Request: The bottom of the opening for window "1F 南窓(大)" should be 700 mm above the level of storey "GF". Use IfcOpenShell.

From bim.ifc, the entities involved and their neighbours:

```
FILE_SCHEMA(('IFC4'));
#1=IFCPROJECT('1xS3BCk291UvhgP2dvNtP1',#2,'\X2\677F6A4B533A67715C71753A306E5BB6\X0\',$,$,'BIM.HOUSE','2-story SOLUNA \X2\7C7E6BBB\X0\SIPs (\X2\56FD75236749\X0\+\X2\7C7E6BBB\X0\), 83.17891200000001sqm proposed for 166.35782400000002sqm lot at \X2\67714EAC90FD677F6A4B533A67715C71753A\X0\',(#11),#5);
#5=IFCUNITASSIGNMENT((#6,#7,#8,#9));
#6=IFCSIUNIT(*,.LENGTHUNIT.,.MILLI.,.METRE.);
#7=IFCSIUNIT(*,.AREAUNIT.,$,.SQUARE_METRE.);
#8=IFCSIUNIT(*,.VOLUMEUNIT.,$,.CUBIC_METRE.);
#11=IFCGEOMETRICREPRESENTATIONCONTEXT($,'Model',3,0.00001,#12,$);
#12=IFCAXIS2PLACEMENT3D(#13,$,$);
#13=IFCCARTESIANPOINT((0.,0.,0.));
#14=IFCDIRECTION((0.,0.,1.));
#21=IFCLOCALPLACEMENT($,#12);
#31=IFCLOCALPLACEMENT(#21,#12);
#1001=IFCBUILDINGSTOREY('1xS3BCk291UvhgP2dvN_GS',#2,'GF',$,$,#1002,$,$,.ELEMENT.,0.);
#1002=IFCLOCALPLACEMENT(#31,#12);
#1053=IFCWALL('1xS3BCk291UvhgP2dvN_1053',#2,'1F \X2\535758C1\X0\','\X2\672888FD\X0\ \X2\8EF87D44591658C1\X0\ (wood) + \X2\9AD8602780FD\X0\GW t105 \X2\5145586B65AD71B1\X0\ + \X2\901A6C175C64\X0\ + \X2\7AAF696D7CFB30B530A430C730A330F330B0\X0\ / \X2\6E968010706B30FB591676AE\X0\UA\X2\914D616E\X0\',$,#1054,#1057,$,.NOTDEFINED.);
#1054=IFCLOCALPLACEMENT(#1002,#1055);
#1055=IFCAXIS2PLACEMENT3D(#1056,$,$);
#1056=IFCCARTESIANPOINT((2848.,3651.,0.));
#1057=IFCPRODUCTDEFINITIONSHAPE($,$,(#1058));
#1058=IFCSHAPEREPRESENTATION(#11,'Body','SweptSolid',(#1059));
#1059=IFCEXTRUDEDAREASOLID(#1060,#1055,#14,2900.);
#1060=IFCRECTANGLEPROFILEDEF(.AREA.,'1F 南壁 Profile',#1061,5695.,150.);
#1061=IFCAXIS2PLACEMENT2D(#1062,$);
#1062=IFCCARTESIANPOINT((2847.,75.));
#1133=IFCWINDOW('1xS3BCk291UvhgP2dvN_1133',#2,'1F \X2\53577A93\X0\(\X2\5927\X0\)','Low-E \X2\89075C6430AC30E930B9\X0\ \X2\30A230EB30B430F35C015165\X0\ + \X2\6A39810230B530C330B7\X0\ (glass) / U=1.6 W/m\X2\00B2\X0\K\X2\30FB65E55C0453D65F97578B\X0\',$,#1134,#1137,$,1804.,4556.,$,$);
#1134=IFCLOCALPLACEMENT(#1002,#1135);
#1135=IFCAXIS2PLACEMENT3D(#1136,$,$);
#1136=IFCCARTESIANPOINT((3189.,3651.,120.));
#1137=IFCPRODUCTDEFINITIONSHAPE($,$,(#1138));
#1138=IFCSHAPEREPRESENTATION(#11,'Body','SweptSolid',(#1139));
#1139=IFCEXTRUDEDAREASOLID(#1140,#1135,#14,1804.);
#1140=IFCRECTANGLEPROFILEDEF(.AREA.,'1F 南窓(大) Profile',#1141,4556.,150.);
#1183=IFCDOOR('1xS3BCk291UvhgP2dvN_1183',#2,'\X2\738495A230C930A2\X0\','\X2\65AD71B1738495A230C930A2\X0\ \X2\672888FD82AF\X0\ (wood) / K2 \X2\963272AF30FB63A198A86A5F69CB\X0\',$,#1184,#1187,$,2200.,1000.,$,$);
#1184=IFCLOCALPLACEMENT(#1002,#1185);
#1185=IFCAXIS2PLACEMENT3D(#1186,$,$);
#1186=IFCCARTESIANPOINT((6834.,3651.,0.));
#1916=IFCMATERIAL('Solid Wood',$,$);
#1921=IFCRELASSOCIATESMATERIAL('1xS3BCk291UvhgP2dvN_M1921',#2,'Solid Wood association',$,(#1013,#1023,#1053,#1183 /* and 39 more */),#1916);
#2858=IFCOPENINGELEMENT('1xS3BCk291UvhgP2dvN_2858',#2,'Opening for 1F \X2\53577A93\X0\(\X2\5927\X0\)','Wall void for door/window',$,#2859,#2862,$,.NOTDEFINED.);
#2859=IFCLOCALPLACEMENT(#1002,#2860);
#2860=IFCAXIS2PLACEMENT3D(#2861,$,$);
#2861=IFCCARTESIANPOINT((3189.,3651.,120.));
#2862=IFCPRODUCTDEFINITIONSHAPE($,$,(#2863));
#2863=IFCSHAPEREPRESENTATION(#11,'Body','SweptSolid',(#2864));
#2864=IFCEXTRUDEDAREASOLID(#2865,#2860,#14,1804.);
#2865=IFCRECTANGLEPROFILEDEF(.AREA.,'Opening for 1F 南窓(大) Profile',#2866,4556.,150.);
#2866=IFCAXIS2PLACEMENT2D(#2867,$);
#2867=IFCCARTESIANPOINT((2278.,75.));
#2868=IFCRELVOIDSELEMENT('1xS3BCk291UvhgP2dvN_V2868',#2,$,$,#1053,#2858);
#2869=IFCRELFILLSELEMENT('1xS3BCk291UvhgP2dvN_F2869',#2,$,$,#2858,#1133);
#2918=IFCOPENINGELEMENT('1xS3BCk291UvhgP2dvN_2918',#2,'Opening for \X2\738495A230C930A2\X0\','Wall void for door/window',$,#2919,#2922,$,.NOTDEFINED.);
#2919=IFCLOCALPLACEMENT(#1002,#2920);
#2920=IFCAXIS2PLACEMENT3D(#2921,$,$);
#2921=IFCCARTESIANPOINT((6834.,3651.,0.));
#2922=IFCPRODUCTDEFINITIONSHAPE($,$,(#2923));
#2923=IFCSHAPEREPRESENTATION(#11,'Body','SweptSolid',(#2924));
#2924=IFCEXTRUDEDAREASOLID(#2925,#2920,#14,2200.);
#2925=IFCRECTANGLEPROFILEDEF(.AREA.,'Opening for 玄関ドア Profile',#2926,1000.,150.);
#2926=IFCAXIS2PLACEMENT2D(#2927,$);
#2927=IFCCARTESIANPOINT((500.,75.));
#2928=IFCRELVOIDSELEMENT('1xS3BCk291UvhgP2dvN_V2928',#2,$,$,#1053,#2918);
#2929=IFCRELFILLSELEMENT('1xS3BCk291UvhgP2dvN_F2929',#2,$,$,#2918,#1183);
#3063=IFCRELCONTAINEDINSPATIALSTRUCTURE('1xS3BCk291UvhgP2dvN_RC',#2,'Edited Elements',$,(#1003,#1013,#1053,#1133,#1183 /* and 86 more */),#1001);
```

```python
import numpy as np
import ifcopenshell
import ifcopenshell.api.geometry
import ifcopenshell.geom
import ifcopenshell.util.element
import ifcopenshell.util.placement
import ifcopenshell.util.shape
import ifcopenshell.util.unit

model = ifcopenshell.open("bim.ifc")
unit_scale = ifcopenshell.util.unit.calculate_unit_scale(model)

window = model.by_guid("1xS3BCk291UvhgP2dvN_1133")
opening = window.FillsVoids[0].RelatingOpeningElement
storey = ifcopenshell.util.element.get_container(window, ifc_class="IfcBuildingStorey")
level = ifcopenshell.util.placement.get_local_placement(storey.ObjectPlacement)[2, 3]

# The opening's origin need not be at the sill, so measure its lowest point.
shape = ifcopenshell.geom.create_shape(ifcopenshell.geom.settings(), opening)
bottom = ifcopenshell.util.shape.get_shape_bottom_elevation(shape, shape.geometry) / unit_scale
dz = level + 700.0 - bottom

shift = np.array([0.0, 0.0, dz])
# The window is not placed relative to its opening, so move both.
for product in (opening, window):
    matrix = ifcopenshell.util.placement.get_local_placement(product.ObjectPlacement)
    matrix[:3, 3] += shift
    ifcopenshell.api.geometry.edit_object_placement(model, product=product, matrix=matrix, is_si=False)

print(f"moved by {dz * unit_scale:+.3f} m")

model.write("bim_rev.ifc")
```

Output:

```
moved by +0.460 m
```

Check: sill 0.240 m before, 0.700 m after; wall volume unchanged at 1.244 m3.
